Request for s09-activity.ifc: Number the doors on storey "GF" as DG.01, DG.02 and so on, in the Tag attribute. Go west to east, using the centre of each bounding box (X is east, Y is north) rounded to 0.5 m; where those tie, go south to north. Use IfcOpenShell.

First a look at what the model holds.

```python
import ifcopenshell
import ifcopenshell.util.element
import ifcopenshell.util.placement

model = ifcopenshell.open("s09-activity.ifc")
print(model.schema)
storey = next(s for s in model.by_type("IfcBuildingStorey") if s.Name == "GF")
doors = [e for e in ifcopenshell.util.element.get_decomposition(storey) if e.is_a("IfcDoor")]
for e in sorted(doors, key=lambda e: e.id()):
    origin = ifcopenshell.util.placement.get_local_placement(e.ObjectPlacement)[:3, 3]
    print(e.id(), e.Tag, e.Name, origin.round(2) + 0.0, sep=" | ")
```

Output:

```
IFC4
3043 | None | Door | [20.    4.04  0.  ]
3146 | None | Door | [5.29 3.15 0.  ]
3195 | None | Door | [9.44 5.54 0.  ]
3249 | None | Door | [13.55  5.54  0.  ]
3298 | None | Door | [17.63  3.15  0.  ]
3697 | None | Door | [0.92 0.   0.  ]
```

```python
import ifcopenshell
import ifcopenshell.geom
import ifcopenshell.util.element
import ifcopenshell.util.shape

model = ifcopenshell.open("s09-activity.ifc")
settings = ifcopenshell.geom.settings()
settings.set("use-world-coords", True)


def centre(element):
    shape = ifcopenshell.geom.create_shape(settings, element)
    return ifcopenshell.util.shape.get_bbox_centroid(shape.geometry)


storey = next(s for s in model.by_type("IfcBuildingStorey") if s.Name == "GF")
doors = [e for e in ifcopenshell.util.element.get_decomposition(storey) if e.is_a("IfcDoor")]

# Insertion points can sit at a corner or the storey origin, so sort by the geometry (in metres).
centres = {e: centre(e) for e in doors}
doors.sort(key=lambda e: (round(centres[e][0] / 0.5), centres[e][1]))

for i, e in enumerate(doors, start=1):
    number = f"DG.{i:02d}"
    e.Tag = number
    print(e.id(), number)

model.write("s09-activity_edited.ifc")
```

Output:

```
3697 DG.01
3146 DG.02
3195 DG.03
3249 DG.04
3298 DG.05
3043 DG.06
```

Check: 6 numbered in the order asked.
